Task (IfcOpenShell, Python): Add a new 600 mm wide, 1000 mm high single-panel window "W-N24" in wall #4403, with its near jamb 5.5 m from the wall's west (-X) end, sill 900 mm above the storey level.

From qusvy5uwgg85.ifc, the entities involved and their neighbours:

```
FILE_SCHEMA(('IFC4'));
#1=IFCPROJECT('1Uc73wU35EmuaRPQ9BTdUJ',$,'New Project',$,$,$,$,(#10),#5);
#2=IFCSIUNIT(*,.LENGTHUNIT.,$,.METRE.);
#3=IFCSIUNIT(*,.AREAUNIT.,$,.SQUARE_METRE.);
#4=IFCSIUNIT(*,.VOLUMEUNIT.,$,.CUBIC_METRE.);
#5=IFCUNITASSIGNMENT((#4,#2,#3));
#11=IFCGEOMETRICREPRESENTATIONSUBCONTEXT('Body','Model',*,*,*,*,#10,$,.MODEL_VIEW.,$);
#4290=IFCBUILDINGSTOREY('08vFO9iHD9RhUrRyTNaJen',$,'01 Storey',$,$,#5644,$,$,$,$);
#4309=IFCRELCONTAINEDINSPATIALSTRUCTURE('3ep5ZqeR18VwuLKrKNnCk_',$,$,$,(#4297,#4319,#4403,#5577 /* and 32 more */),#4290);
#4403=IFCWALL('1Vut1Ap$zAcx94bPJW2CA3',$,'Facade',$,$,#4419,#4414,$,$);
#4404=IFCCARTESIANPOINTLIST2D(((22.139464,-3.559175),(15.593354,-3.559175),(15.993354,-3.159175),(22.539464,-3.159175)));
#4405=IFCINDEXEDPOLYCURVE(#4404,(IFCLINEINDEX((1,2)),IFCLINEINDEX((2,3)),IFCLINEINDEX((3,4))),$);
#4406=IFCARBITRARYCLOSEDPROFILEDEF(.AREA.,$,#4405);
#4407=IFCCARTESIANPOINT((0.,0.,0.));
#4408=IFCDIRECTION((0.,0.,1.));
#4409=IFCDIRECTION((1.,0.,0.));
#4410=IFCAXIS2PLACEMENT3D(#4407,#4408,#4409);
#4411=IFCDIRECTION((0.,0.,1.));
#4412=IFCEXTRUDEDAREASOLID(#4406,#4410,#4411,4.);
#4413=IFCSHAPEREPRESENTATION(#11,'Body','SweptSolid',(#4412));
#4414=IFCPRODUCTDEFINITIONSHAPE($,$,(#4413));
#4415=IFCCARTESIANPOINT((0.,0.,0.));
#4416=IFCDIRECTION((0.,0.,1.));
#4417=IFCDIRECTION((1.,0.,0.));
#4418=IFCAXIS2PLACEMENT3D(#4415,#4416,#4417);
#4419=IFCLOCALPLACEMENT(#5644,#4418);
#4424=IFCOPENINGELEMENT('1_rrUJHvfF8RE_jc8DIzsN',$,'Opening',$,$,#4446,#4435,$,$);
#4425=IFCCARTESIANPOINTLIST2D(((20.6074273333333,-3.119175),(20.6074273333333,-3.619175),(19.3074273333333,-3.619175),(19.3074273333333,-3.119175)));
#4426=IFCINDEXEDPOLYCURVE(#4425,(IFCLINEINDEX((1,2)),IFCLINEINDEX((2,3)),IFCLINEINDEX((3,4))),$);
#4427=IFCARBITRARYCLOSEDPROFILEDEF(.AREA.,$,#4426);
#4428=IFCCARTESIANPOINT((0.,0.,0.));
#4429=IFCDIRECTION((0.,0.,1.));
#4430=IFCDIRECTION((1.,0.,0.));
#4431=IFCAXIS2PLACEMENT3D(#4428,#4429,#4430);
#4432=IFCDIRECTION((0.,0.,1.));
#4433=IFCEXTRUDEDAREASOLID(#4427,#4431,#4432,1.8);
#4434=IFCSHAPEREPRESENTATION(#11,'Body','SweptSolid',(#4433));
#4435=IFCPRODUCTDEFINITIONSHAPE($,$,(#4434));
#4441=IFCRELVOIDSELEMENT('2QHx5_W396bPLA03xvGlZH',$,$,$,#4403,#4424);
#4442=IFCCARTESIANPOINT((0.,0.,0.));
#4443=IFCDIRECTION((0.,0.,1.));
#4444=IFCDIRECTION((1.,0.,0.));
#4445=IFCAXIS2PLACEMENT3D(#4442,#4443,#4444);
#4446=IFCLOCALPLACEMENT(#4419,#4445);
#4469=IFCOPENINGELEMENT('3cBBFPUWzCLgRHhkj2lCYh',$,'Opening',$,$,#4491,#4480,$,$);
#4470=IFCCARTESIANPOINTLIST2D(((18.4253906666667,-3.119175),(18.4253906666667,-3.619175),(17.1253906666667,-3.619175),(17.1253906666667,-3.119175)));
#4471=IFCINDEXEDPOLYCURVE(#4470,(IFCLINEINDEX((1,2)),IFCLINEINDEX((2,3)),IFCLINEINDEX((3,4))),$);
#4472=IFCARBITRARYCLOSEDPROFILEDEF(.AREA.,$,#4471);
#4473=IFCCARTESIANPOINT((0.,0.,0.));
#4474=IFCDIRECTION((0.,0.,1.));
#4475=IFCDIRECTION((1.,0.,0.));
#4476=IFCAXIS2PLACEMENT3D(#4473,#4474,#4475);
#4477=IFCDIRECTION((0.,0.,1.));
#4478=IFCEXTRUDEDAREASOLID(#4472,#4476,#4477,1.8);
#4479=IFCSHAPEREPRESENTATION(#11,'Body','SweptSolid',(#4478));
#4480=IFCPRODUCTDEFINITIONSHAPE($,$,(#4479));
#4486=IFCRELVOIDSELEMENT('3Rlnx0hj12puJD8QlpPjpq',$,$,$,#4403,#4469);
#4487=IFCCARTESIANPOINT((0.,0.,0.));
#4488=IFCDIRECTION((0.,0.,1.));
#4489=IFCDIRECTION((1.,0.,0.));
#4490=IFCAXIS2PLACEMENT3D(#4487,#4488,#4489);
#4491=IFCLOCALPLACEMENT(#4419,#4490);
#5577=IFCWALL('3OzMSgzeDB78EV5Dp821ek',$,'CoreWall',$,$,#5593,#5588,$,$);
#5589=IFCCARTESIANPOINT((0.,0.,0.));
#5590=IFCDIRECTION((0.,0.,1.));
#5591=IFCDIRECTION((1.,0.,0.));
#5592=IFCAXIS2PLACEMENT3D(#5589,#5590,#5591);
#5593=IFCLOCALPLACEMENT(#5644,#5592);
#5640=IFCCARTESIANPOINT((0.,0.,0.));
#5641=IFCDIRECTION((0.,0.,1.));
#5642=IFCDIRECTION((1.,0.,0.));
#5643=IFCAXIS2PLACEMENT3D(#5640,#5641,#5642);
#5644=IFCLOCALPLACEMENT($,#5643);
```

```python
import numpy as np
import ifcopenshell
import ifcopenshell.api.feature
import ifcopenshell.api.geometry
import ifcopenshell.api.root
import ifcopenshell.api.spatial
import ifcopenshell.geom
import ifcopenshell.util.element
import ifcopenshell.util.placement
import ifcopenshell.util.representation
import ifcopenshell.util.shape
import ifcopenshell.util.unit

model = ifcopenshell.open("qusvy5uwgg85.ifc")
unit_scale = ifcopenshell.util.unit.calculate_unit_scale(model)
settings = ifcopenshell.geom.settings()


def volume(element):
    """Net volume in cubic metres, openings subtracted."""
    shape = ifcopenshell.geom.create_shape(settings, element)
    return ifcopenshell.util.shape.get_volume(shape.geometry)


wall = model.by_id(4403)
storey = ifcopenshell.util.element.get_container(wall, ifc_class="IfcBuildingStorey")
context = ifcopenshell.util.representation.get_context(model, "Model", "Body", "MODEL_VIEW")
before = volume(wall)

width, height, from_end, sill = 0.6, 1, 5.5, 0.9  # metres

# The wall runs along its own X axis, and the end named is its -X end.
wall_shape = ifcopenshell.geom.create_shape(settings, wall)
x, y, z = ifcopenshell.util.shape.get_vertices(wall_shape.geometry).T
start = x.min() + from_end
face, thickness = float(y.min()), float(y.max() - y.min())
wall_matrix = ifcopenshell.util.placement.get_local_placement(wall.ObjectPlacement)
level = ifcopenshell.util.placement.get_local_placement(storey.ObjectPlacement)[2, 3]


def in_wall(x, y):
    """Placement at x, y metres in the wall's axes, at sill height."""
    matrix = wall_matrix.copy()
    matrix[:, 3] = wall_matrix @ np.array([x / unit_scale, y / unit_scale, 0.0, 1.0])
    matrix[2, 3] = level + sill / unit_scale
    return matrix


# Opening: a box that overshoots both wall faces by 50 mm.
opening = ifcopenshell.api.root.create_entity(model, ifc_class="IfcOpeningElement", predefined_type="OPENING")
box = ifcopenshell.api.geometry.add_wall_representation(
    model, context=context, length=width, height=height, thickness=thickness + 0.1
)
ifcopenshell.api.geometry.assign_representation(model, product=opening, representation=box)
ifcopenshell.api.geometry.edit_object_placement(model, product=opening, matrix=in_wall(start, face - 0.05), is_si=False)
ifcopenshell.api.feature.add_feature(model, feature=opening, element=wall)

window = ifcopenshell.api.root.create_entity(model, ifc_class="IfcWindow", name="W-N24", predefined_type="WINDOW")
window.OverallWidth, window.OverallHeight = width / unit_scale, height / unit_scale
window.PartitioningType = "SINGLE_PANEL"
body = ifcopenshell.api.geometry.add_window_representation(
    model,
    context=context,
    overall_width=window.OverallWidth,
    overall_height=window.OverallHeight,
    partition_type="SINGLE_PANEL",
)
ifcopenshell.api.geometry.assign_representation(model, product=window, representation=body)
ifcopenshell.api.spatial.assign_container(model, products=[window], relating_structure=storey)
ifcopenshell.api.feature.add_filling(model, opening=opening, element=window)

# Centre the window in the wall's thickness.
ifcopenshell.api.geometry.edit_object_placement(model, product=window, matrix=in_wall(start, face), is_si=False)
window_shape = ifcopenshell.geom.create_shape(settings, window)
depth = ifcopenshell.util.shape.get_vertices(window_shape.geometry)[:, 1]
offset = face + thickness / 2 - (depth.min() + depth.max()) / 2
ifcopenshell.api.geometry.edit_object_placement(model, product=window, matrix=in_wall(start, offset), is_si=False)

after = volume(wall)

print(f"wall volume {before:.3f} -> {after:.3f} m3")

model.write("qusvy5uwgg85_updated.ifc")
```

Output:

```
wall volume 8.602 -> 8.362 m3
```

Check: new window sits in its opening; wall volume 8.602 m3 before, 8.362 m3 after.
